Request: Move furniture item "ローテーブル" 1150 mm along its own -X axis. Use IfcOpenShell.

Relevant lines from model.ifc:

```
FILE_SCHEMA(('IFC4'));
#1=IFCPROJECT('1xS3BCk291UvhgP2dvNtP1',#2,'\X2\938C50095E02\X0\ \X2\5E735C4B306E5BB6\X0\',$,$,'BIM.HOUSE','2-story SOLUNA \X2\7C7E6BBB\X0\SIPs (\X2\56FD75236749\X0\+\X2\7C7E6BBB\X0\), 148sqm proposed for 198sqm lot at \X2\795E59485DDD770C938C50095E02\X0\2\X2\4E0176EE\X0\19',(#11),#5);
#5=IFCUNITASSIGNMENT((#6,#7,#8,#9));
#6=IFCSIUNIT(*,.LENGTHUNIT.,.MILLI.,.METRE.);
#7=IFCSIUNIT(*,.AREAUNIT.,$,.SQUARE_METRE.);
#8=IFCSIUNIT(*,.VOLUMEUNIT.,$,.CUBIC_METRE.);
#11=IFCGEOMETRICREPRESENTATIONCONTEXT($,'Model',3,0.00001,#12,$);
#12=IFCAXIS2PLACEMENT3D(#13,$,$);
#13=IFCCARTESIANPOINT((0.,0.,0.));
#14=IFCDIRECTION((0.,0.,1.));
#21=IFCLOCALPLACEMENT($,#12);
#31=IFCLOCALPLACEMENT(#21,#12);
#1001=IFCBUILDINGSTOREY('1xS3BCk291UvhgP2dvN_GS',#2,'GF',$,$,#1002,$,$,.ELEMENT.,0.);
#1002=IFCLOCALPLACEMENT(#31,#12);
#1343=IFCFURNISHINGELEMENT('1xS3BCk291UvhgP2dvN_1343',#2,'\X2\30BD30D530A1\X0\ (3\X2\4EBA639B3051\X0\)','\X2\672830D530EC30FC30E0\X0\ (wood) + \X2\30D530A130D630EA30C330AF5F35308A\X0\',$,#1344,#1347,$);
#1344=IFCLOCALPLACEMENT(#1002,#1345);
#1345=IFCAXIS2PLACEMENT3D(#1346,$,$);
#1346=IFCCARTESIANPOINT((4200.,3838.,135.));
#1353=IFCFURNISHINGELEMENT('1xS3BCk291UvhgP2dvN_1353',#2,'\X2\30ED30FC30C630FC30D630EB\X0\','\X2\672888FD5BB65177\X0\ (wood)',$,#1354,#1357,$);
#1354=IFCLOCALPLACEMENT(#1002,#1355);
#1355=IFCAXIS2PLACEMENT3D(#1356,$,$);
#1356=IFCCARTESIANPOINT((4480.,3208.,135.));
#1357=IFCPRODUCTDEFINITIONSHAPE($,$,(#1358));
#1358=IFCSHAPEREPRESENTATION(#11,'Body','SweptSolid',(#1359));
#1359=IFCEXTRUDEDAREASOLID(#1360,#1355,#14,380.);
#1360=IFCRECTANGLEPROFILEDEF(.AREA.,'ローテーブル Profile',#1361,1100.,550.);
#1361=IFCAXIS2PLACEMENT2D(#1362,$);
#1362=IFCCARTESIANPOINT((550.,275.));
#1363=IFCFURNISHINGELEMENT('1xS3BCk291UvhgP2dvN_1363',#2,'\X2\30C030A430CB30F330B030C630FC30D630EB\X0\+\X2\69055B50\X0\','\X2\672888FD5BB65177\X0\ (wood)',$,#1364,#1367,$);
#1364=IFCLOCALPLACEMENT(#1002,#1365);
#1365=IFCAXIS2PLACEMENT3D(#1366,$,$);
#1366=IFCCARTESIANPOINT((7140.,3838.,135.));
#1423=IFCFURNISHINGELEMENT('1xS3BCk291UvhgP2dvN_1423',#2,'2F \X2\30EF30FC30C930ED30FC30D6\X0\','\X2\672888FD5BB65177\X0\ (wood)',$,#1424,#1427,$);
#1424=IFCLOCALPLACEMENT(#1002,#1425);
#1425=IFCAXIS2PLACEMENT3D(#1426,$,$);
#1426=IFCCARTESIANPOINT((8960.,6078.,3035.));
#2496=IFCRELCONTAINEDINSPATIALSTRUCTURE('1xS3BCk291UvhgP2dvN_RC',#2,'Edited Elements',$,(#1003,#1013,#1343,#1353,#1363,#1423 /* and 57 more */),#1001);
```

```python
import ifcopenshell
import ifcopenshell.api.geometry
import ifcopenshell.util.placement
import ifcopenshell.util.unit

model = ifcopenshell.open("model.ifc")
unit_scale = ifcopenshell.util.unit.calculate_unit_scale(model)

item = model.by_guid("1xS3BCk291UvhgP2dvN_1353")
matrix = ifcopenshell.util.placement.get_local_placement(item.ObjectPlacement)
matrix[:3, 3] -= matrix[:3, 0] * 1.15 / unit_scale
ifcopenshell.api.geometry.edit_object_placement(model, product=item, matrix=matrix, is_si=False)

print(ifcopenshell.util.placement.get_local_placement(item.ObjectPlacement).round(3) + 0.0)

model.write("model_rev.ifc")
```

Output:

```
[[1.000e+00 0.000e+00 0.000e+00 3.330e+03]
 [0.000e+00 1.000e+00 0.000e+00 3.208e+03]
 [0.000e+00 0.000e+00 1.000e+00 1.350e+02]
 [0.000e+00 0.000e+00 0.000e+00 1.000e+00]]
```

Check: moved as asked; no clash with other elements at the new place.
